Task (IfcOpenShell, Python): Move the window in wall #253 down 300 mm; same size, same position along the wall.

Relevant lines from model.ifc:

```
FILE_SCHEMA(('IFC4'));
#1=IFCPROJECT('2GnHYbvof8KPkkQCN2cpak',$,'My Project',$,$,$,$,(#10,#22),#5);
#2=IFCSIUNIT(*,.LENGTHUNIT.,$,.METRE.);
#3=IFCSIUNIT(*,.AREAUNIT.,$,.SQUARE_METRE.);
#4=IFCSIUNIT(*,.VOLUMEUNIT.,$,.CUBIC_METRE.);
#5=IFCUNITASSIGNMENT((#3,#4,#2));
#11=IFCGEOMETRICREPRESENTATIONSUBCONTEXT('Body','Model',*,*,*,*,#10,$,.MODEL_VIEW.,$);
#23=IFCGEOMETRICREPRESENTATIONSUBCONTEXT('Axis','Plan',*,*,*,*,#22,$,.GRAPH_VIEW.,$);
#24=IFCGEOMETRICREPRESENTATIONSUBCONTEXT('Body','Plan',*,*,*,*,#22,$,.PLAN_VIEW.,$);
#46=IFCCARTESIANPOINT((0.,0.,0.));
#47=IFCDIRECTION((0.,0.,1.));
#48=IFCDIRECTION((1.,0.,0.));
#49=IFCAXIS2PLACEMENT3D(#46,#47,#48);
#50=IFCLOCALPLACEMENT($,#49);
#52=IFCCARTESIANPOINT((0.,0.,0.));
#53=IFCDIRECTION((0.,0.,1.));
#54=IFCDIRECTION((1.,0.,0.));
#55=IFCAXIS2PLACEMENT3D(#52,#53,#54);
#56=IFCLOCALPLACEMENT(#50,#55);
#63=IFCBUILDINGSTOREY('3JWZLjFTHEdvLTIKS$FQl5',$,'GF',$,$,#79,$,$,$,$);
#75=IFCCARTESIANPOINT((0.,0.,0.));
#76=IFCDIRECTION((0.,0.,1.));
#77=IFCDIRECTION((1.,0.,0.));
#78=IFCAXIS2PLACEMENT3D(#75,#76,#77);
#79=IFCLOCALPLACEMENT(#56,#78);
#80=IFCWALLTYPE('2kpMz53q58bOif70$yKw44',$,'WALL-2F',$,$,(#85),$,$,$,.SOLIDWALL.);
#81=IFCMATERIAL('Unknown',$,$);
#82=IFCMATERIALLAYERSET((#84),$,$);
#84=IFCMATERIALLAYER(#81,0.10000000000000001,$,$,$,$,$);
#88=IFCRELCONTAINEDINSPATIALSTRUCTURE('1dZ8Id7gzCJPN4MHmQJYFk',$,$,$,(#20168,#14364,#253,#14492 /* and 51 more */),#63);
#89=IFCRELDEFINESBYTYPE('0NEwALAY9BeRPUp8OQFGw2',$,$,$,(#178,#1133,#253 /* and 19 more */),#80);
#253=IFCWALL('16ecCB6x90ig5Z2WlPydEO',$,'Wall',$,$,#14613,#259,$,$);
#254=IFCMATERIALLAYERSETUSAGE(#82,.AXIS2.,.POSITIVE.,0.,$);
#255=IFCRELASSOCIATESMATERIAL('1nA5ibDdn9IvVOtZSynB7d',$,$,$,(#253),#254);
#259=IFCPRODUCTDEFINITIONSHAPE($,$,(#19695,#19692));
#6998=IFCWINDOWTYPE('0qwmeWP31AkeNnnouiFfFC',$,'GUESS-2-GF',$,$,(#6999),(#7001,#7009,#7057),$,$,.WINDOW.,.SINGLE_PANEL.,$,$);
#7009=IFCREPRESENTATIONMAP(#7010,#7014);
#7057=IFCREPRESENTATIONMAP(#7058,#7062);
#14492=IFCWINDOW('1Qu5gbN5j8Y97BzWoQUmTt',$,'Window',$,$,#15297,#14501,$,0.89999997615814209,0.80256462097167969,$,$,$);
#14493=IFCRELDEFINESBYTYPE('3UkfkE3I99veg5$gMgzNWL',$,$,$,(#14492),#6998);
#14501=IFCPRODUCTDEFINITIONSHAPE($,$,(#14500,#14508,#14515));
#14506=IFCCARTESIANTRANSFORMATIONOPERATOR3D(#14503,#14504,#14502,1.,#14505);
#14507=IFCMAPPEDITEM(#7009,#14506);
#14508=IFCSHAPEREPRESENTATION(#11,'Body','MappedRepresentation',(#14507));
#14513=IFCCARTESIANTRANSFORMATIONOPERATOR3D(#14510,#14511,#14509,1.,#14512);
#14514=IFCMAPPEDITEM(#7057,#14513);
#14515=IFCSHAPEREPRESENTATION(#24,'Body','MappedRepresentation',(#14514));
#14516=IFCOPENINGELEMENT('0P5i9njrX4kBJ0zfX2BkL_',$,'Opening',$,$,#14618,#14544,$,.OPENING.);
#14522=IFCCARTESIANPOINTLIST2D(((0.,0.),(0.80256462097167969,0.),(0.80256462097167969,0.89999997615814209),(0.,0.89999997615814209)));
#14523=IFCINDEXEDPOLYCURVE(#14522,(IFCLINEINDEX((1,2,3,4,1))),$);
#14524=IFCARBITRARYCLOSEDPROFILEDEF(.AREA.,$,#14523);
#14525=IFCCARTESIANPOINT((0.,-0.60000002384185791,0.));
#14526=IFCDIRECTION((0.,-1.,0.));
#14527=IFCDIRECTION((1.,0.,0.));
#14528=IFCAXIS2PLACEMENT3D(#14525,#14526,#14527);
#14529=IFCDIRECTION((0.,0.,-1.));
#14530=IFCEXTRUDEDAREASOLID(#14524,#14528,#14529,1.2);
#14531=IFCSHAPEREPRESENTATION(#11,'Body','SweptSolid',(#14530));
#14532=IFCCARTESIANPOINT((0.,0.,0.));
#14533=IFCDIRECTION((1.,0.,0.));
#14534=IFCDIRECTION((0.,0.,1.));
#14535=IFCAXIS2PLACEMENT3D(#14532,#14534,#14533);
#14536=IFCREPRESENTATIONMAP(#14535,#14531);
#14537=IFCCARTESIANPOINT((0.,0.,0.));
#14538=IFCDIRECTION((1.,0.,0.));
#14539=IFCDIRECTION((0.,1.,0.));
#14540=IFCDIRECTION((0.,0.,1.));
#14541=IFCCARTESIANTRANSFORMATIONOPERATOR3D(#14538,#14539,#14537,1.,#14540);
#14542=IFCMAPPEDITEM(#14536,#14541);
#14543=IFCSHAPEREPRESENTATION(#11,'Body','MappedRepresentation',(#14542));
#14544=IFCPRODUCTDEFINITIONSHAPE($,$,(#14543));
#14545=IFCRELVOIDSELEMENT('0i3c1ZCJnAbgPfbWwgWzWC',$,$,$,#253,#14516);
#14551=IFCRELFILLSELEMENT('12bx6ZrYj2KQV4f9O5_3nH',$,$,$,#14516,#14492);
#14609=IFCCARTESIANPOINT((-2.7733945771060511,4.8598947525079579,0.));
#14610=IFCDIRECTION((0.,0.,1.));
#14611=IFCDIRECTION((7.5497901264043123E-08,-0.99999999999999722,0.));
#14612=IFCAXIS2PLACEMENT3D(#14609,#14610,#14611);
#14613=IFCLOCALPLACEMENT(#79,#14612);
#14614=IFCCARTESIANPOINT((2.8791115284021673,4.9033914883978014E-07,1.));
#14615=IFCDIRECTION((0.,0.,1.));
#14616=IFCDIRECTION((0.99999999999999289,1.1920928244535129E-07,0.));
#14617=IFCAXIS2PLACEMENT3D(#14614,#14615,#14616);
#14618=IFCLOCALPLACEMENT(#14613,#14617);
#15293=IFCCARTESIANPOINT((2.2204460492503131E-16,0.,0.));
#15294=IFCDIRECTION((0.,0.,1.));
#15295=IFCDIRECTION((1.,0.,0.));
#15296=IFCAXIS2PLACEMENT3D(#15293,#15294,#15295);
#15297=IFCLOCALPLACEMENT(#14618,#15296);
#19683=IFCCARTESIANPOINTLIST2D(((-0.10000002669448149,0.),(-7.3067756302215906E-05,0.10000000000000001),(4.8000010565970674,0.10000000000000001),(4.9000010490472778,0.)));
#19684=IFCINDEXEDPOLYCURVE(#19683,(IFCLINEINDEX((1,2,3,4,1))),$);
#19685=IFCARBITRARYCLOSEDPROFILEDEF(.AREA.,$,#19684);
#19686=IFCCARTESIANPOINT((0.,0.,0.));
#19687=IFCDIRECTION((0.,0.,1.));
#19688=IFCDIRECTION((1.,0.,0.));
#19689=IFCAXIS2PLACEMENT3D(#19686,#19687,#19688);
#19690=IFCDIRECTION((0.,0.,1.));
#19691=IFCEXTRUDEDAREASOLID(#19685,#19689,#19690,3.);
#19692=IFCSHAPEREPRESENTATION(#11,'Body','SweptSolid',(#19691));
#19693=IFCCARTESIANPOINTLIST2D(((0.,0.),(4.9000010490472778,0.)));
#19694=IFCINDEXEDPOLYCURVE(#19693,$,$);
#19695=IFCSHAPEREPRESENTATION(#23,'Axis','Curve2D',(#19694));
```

```python
import numpy as np
import ifcopenshell
import ifcopenshell.api.geometry
import ifcopenshell.util.placement
import ifcopenshell.util.unit

model = ifcopenshell.open("model.ifc")
unit_scale = ifcopenshell.util.unit.calculate_unit_scale(model)

window = model.by_guid("1Qu5gbN5j8Y97BzWoQUmTt")
opening = window.FillsVoids[0].RelatingOpeningElement
dz = -0.3 / unit_scale

shift = np.array([0.0, 0.0, dz])
# The window is placed relative to its opening, so it follows when the opening moves.
matrix = ifcopenshell.util.placement.get_local_placement(opening.ObjectPlacement)
matrix[:3, 3] += shift
ifcopenshell.api.geometry.edit_object_placement(
    model, product=opening, matrix=matrix, is_si=False, should_transform_children=True
)

print(f"moved by {dz * unit_scale:+.3f} m")

model.write("model_updated.ifc")
```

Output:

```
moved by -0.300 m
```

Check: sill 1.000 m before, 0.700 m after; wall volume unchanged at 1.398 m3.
